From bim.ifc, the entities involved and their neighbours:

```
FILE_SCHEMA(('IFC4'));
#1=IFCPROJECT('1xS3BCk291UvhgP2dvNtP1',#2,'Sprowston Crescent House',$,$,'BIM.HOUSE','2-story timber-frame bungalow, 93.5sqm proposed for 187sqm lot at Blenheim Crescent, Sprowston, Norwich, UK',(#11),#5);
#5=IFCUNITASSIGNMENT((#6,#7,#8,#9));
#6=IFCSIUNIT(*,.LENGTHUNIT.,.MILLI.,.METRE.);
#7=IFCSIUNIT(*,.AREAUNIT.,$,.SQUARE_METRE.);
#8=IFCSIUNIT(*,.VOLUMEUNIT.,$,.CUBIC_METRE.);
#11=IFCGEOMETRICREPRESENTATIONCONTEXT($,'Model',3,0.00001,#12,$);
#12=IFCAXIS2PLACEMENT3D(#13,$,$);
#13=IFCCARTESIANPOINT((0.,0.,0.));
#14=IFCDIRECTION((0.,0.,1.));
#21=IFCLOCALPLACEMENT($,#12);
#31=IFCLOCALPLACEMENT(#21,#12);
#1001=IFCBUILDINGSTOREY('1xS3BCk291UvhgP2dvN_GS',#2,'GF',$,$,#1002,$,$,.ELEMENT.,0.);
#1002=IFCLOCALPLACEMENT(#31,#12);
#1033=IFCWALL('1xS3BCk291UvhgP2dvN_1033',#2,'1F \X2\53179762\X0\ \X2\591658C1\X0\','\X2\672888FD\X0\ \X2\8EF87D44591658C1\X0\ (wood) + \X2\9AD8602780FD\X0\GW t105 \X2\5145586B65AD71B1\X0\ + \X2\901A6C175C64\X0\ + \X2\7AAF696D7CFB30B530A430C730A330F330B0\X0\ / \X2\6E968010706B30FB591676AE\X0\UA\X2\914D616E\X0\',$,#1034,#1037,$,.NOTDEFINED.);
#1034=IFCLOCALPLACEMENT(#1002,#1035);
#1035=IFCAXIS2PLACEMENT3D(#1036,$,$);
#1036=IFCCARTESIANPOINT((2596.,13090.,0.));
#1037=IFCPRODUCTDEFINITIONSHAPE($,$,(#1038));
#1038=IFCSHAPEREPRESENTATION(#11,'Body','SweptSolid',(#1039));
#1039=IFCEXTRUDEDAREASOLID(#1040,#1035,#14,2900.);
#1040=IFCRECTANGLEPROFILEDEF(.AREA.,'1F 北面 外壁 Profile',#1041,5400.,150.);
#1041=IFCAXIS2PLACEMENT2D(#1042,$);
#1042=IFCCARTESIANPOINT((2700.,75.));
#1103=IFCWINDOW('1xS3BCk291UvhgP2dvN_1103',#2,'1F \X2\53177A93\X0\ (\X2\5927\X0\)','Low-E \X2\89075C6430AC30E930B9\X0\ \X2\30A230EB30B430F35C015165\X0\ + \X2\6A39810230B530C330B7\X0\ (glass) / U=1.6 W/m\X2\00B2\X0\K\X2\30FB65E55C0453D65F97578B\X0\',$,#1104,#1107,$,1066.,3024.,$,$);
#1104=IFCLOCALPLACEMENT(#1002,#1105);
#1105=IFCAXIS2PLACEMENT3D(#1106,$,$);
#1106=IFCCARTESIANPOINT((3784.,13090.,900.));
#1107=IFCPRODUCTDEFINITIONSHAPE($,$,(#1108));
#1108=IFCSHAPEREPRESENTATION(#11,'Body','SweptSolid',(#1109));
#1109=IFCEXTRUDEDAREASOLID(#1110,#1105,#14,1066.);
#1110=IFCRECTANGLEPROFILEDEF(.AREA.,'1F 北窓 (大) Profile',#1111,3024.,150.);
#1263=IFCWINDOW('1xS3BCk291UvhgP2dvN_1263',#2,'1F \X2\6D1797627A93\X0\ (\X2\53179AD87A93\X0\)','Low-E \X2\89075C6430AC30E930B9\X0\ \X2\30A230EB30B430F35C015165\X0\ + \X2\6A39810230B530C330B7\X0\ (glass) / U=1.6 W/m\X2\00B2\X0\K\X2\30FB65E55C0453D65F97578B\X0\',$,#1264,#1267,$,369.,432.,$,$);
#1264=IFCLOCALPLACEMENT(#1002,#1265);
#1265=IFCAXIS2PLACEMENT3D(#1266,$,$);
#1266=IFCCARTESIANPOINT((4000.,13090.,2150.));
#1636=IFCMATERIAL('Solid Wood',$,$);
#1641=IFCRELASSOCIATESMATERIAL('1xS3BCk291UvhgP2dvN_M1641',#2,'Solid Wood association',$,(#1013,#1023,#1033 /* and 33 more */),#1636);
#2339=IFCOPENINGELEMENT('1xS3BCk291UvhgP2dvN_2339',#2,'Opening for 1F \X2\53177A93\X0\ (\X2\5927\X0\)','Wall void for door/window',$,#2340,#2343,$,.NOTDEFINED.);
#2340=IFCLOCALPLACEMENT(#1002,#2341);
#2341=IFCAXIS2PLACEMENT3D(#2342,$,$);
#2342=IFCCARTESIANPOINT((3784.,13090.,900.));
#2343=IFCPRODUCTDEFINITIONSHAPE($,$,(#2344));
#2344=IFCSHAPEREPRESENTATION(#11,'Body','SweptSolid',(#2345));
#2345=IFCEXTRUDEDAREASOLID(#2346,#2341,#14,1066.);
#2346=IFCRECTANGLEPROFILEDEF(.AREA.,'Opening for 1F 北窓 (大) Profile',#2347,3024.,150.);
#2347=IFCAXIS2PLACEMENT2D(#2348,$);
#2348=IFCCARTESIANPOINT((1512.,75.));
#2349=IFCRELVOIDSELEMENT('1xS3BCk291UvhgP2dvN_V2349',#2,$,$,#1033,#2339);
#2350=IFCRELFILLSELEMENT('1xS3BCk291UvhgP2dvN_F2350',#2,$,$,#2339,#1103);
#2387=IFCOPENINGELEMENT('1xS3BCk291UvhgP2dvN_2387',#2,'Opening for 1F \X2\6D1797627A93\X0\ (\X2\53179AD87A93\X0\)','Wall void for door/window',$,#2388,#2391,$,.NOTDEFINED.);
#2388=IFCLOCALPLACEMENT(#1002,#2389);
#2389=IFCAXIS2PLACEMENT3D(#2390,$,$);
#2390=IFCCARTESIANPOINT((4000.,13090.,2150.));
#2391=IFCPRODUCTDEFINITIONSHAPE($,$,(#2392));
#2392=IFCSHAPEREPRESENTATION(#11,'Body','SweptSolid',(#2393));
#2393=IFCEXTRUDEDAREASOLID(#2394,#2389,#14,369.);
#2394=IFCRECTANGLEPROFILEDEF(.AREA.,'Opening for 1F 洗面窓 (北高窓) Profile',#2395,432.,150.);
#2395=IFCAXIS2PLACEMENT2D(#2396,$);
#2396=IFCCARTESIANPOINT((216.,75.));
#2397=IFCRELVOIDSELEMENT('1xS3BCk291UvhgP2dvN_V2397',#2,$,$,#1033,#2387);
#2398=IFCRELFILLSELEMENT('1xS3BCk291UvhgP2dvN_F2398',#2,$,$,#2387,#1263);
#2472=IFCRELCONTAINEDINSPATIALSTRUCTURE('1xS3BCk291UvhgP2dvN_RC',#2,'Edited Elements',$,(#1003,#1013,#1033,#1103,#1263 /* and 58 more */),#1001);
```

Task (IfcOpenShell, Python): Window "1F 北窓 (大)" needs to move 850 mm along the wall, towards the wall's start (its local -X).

```python
import ifcopenshell
import ifcopenshell.api.geometry
import ifcopenshell.util.placement
import ifcopenshell.util.unit

model = ifcopenshell.open("bim.ifc")
unit_scale = ifcopenshell.util.unit.calculate_unit_scale(model)

window = model.by_guid("1xS3BCk291UvhgP2dvN_1103")
opening = window.FillsVoids[0].RelatingOpeningElement
wall = opening.VoidsElements[0].RelatingBuildingElement

wall_matrix = ifcopenshell.util.placement.get_local_placement(wall.ObjectPlacement)
shift = wall_matrix[:3, 0] * -0.85 / unit_scale
before = ifcopenshell.util.placement.get_local_placement(window.ObjectPlacement)[:3, 3].copy()

# The window is not placed relative to its opening, so move both.
for product in (opening, window):
    matrix = ifcopenshell.util.placement.get_local_placement(product.ObjectPlacement)
    matrix[:3, 3] += shift
    ifcopenshell.api.geometry.edit_object_placement(model, product=product, matrix=matrix, is_si=False)

after = ifcopenshell.util.placement.get_local_placement(window.ObjectPlacement)[:3, 3]
print("window moved by", (after - before).round(3) + 0.0)

model.write("bim-out.ifc")
```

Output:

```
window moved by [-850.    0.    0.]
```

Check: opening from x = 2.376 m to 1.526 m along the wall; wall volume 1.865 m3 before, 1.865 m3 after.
